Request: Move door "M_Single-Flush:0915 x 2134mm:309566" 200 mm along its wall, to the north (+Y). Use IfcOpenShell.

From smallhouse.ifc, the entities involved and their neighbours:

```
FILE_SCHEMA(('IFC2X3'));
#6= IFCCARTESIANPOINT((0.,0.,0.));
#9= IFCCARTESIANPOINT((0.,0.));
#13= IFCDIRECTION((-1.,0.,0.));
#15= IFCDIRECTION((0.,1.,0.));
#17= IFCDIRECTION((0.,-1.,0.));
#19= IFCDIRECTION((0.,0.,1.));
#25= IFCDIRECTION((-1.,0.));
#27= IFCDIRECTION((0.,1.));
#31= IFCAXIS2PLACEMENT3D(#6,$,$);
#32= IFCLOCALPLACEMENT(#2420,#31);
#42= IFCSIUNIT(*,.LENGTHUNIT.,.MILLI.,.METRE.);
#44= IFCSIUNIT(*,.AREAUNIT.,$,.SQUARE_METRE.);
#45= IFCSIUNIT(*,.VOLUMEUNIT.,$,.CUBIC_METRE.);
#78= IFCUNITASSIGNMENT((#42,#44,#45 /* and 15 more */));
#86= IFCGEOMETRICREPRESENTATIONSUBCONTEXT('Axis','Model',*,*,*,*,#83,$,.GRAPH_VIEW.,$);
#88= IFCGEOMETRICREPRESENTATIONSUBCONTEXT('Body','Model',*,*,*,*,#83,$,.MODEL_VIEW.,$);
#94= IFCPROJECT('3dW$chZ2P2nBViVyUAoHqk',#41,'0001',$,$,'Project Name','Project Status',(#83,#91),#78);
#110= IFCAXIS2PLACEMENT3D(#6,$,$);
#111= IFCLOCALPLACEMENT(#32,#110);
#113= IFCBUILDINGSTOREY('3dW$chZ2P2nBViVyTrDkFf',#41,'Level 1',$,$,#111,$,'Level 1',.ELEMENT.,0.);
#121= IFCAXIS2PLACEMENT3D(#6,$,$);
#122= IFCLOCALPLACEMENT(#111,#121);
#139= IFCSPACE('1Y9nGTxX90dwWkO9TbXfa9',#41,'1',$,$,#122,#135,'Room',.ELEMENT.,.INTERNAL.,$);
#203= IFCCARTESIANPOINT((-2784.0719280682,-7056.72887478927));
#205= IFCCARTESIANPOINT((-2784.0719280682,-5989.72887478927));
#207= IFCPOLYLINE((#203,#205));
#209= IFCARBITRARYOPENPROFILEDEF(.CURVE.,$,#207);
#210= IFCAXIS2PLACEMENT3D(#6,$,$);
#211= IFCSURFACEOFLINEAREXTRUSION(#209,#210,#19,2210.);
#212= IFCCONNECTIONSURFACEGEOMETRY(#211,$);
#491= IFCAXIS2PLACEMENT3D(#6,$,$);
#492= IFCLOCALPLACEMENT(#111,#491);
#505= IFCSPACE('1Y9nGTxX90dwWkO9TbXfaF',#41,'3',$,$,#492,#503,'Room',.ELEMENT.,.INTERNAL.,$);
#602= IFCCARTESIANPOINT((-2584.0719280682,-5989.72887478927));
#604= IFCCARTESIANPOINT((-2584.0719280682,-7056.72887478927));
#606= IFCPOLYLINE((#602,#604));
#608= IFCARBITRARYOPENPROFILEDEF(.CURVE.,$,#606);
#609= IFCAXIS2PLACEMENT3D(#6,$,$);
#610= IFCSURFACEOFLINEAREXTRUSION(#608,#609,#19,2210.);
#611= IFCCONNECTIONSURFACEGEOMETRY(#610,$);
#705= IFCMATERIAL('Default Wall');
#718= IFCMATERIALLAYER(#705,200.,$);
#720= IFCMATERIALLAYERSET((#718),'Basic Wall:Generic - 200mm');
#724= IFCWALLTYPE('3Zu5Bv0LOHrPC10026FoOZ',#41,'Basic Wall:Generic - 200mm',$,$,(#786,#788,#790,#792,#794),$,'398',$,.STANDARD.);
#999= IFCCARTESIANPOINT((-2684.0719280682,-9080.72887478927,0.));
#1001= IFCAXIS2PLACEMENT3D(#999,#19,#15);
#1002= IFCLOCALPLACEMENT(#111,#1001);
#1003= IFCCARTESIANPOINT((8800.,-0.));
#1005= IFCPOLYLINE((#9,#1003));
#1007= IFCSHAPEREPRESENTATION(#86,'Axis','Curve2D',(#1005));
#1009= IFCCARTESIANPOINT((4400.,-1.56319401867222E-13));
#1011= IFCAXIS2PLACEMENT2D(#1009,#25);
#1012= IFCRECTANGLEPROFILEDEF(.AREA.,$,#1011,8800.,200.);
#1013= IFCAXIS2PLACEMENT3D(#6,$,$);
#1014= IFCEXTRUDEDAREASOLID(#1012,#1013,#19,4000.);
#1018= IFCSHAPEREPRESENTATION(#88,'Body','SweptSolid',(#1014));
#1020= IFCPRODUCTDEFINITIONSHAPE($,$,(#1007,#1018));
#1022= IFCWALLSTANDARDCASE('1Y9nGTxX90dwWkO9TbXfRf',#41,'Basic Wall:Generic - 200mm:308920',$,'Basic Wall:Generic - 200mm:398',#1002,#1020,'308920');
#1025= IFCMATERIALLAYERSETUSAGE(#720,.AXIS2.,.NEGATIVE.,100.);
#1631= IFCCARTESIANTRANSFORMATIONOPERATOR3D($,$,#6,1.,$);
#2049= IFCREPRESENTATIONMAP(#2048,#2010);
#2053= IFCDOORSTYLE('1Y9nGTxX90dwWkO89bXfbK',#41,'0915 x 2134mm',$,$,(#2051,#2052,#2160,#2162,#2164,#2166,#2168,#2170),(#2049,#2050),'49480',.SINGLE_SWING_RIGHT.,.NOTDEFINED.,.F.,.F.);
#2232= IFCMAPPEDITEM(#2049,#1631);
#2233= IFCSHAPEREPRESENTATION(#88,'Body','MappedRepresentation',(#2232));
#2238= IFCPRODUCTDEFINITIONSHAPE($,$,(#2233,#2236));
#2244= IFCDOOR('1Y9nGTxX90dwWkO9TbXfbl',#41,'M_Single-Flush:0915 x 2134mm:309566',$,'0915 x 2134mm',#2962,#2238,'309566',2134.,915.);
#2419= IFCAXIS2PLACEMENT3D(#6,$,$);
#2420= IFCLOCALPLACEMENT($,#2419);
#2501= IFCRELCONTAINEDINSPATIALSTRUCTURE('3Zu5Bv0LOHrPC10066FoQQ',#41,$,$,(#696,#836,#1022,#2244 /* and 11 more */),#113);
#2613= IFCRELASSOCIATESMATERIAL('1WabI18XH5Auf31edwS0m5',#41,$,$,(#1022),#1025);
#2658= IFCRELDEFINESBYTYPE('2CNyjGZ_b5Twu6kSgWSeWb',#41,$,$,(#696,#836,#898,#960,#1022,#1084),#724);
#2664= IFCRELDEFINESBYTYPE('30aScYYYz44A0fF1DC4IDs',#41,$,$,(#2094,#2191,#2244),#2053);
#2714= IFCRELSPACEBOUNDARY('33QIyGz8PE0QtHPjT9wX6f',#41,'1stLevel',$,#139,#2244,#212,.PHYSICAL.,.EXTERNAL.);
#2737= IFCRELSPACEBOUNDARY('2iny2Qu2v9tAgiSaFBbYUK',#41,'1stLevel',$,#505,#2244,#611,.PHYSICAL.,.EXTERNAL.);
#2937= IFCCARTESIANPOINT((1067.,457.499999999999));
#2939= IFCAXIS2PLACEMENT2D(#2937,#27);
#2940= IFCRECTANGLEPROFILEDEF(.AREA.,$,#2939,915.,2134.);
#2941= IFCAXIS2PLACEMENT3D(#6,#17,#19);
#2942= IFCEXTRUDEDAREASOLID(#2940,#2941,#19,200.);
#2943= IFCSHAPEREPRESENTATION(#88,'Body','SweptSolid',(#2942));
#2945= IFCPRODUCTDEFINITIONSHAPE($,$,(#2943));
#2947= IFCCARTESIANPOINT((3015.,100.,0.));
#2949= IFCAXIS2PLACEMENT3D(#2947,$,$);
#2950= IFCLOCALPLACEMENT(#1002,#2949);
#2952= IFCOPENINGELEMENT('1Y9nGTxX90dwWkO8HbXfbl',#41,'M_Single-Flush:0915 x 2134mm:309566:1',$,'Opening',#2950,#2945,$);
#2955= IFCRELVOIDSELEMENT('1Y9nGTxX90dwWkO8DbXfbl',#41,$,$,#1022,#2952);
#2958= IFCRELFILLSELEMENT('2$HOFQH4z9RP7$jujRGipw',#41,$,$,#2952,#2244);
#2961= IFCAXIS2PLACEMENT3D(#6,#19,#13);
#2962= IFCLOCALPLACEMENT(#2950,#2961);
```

```python
import numpy as np
import ifcopenshell
import ifcopenshell.api.geometry
import ifcopenshell.util.placement
import ifcopenshell.util.unit

model = ifcopenshell.open("smallhouse.ifc")
unit_scale = ifcopenshell.util.unit.calculate_unit_scale(model)

door = model.by_guid("1Y9nGTxX90dwWkO9TbXfbl")
opening = door.FillsVoids[0].RelatingOpeningElement
wall = opening.VoidsElements[0].RelatingBuildingElement

wall_matrix = ifcopenshell.util.placement.get_local_placement(wall.ObjectPlacement)
shift = wall_matrix[:3, 0] * 0.2 / unit_scale
before = ifcopenshell.util.placement.get_local_placement(door.ObjectPlacement)[:3, 3].copy()

# The door is placed relative to its opening, so it follows when the opening moves.
matrix = ifcopenshell.util.placement.get_local_placement(opening.ObjectPlacement)
matrix[:3, 3] += shift
ifcopenshell.api.geometry.edit_object_placement(
    model, product=opening, matrix=matrix, is_si=False, should_transform_children=True
)

# Space boundary surfaces are stored in each space's coordinates; move them too.
for rel in door.ProvidesBoundaries:
    if not rel.ConnectionGeometry:
        continue
    surface = rel.ConnectionGeometry.SurfaceOnRelatingElement
    space_matrix = ifcopenshell.util.placement.get_local_placement(rel.RelatingSpace.ObjectPlacement)
    point = np.array(surface.Position.Location.Coordinates) + space_matrix[:3, :3].T @ shift
    surface.Position = model.createIfcAxis2Placement3D(
        model.createIfcCartesianPoint(point.tolist()), surface.Position.Axis, surface.Position.RefDirection
    )

after = ifcopenshell.util.placement.get_local_placement(door.ObjectPlacement)[:3, 3]
print("door moved by", (after - before).round(3) + 0.0)

model.write("smallhouse_rev.ifc")
```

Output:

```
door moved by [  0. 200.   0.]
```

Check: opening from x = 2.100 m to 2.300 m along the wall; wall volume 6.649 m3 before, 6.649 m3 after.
